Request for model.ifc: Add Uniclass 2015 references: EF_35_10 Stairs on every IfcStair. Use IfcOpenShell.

First a look at what the model holds.

```python
import ifcopenshell

model = ifcopenshell.open("model.ifc")
print(model.schema)
print("classifications:", [c.Name for c in model.by_type("IfcClassification")])
for ifc_class in ("IfcDoor", "IfcRoof", "IfcStair", "IfcWall", "IfcWindow"):
    print(ifc_class, len(model.by_type(ifc_class)))
```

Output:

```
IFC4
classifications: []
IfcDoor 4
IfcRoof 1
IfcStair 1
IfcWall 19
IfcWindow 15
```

```python
import ifcopenshell
import ifcopenshell.api.classification

model = ifcopenshell.open("model.ifc")

system = ifcopenshell.api.classification.add_classification(model, classification="Uniclass 2015")

codes = {
    "IfcStair": ("EF_35_10", "Stairs"),
}
for ifc_class, (code, name) in codes.items():
    products = model.by_type(ifc_class)
    ifcopenshell.api.classification.add_reference(
        model, products=products, classification=system, identification=code, name=name
    )
    print(code, len(products))

model.write("model_edited.ifc")
```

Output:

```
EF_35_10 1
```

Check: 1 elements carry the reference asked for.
